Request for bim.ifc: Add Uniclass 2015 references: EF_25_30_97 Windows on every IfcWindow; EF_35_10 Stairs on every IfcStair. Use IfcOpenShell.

First a look at what the model holds.

```python
import ifcopenshell

model = ifcopenshell.open("bim.ifc")
print(model.schema)
print("classifications:", [c.Name for c in model.by_type("IfcClassification")])
for ifc_class in ("IfcDoor", "IfcRoof", "IfcStair", "IfcWall", "IfcWindow"):
    print(ifc_class, len(model.by_type(ifc_class)))
```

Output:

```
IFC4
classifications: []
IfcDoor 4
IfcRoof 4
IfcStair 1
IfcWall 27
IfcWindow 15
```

```python
import ifcopenshell
import ifcopenshell.api.classification

model = ifcopenshell.open("bim.ifc")

system = ifcopenshell.api.classification.add_classification(model, classification="Uniclass 2015")

codes = {
    "IfcWindow": ("EF_25_30_97", "Windows"),
    "IfcStair": ("EF_35_10", "Stairs"),
}
for ifc_class, (code, name) in codes.items():
    products = model.by_type(ifc_class)
    ifcopenshell.api.classification.add_reference(
        model, products=products, classification=system, identification=code, name=name
    )
    print(code, len(products))

model.write("bim-out.ifc")
```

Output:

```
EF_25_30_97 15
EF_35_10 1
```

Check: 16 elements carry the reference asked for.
